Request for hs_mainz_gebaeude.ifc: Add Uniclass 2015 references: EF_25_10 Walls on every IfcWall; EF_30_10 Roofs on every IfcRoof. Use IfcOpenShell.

First a look at what the model holds.

```python
import ifcopenshell

model = ifcopenshell.open("hs_mainz_gebaeude.ifc")
print(model.schema)
print("classifications:", [c.Name for c in model.by_type("IfcClassification")])
for ifc_class in ("IfcDoor", "IfcRoof", "IfcStair", "IfcWall", "IfcWindow"):
    print(ifc_class, len(model.by_type(ifc_class)))
```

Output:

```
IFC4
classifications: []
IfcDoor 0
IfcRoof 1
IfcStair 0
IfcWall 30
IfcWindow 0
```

```python
import ifcopenshell
import ifcopenshell.api.classification

model = ifcopenshell.open("hs_mainz_gebaeude.ifc")

system = ifcopenshell.api.classification.add_classification(model, classification="Uniclass 2015")

codes = {
    "IfcWall": ("EF_25_10", "Walls"),
    "IfcRoof": ("EF_30_10", "Roofs"),
}
for ifc_class, (code, name) in codes.items():
    products = model.by_type(ifc_class)
    ifcopenshell.api.classification.add_reference(
        model, products=products, classification=system, identification=code, name=name
    )
    print(code, len(products))

model.write("hs_mainz_gebaeude_rev.ifc")
```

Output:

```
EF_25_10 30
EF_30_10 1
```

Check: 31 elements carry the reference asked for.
